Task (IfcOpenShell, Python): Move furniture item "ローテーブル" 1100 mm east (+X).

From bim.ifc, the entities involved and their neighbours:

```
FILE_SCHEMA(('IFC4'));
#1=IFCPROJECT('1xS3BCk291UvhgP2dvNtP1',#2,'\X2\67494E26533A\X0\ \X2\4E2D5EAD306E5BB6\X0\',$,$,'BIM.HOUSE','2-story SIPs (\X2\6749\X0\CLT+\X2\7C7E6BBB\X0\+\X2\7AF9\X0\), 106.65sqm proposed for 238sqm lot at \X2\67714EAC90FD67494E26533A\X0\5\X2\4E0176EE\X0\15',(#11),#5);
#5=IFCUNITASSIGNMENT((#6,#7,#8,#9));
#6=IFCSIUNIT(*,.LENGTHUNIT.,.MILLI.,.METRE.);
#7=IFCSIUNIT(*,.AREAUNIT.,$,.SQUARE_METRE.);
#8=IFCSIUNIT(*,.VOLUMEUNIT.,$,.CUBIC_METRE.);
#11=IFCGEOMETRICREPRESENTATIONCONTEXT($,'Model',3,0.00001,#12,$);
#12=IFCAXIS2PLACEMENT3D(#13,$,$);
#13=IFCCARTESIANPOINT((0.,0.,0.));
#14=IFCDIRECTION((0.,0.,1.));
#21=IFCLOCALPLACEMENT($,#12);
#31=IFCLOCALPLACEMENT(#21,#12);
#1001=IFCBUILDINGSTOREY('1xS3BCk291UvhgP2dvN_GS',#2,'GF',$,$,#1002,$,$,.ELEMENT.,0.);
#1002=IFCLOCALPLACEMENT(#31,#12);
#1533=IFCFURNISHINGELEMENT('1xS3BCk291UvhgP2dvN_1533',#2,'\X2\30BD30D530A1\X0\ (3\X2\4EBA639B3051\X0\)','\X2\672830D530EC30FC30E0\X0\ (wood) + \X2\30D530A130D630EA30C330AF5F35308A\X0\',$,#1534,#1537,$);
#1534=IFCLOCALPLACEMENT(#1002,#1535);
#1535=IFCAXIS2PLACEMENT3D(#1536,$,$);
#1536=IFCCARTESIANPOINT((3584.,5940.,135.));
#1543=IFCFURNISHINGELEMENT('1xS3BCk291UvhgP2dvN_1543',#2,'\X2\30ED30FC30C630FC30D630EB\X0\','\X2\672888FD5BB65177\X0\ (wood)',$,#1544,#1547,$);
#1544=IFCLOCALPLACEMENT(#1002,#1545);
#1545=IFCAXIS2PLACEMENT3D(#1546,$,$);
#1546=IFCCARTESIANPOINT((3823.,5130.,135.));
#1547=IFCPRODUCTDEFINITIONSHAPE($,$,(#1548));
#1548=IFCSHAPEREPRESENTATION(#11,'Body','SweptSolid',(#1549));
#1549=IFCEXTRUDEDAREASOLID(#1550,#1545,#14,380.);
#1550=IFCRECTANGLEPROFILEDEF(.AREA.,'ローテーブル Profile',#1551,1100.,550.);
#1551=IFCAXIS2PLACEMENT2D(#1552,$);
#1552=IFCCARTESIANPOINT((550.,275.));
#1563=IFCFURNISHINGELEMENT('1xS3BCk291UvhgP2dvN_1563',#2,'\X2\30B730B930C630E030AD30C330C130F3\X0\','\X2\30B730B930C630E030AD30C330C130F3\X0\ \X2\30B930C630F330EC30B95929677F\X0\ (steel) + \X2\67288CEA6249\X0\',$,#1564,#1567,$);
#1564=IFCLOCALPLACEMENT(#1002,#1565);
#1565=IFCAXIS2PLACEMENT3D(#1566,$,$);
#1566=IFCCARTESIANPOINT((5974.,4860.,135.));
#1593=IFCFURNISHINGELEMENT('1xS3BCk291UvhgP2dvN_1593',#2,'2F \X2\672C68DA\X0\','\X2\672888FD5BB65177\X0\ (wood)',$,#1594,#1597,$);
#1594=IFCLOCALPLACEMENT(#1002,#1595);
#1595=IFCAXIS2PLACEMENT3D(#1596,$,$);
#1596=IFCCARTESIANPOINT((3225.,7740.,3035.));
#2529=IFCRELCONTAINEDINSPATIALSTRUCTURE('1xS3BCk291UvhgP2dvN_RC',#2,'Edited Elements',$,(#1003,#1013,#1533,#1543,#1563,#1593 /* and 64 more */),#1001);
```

```python
import ifcopenshell
import ifcopenshell.api.geometry
import ifcopenshell.util.placement
import ifcopenshell.util.unit

model = ifcopenshell.open("bim.ifc")
unit_scale = ifcopenshell.util.unit.calculate_unit_scale(model)

item = model.by_guid("1xS3BCk291UvhgP2dvN_1543")
matrix = ifcopenshell.util.placement.get_local_placement(item.ObjectPlacement)
matrix[0, 3] += 1.1 / unit_scale
ifcopenshell.api.geometry.edit_object_placement(model, product=item, matrix=matrix, is_si=False)

print(ifcopenshell.util.placement.get_local_placement(item.ObjectPlacement).round(3) + 0.0)

model.write("bim_updated.ifc")
```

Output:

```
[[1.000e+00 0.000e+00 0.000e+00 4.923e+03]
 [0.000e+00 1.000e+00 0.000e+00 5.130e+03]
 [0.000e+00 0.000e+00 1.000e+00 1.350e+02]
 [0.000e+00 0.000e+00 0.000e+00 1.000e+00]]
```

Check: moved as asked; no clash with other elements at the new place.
